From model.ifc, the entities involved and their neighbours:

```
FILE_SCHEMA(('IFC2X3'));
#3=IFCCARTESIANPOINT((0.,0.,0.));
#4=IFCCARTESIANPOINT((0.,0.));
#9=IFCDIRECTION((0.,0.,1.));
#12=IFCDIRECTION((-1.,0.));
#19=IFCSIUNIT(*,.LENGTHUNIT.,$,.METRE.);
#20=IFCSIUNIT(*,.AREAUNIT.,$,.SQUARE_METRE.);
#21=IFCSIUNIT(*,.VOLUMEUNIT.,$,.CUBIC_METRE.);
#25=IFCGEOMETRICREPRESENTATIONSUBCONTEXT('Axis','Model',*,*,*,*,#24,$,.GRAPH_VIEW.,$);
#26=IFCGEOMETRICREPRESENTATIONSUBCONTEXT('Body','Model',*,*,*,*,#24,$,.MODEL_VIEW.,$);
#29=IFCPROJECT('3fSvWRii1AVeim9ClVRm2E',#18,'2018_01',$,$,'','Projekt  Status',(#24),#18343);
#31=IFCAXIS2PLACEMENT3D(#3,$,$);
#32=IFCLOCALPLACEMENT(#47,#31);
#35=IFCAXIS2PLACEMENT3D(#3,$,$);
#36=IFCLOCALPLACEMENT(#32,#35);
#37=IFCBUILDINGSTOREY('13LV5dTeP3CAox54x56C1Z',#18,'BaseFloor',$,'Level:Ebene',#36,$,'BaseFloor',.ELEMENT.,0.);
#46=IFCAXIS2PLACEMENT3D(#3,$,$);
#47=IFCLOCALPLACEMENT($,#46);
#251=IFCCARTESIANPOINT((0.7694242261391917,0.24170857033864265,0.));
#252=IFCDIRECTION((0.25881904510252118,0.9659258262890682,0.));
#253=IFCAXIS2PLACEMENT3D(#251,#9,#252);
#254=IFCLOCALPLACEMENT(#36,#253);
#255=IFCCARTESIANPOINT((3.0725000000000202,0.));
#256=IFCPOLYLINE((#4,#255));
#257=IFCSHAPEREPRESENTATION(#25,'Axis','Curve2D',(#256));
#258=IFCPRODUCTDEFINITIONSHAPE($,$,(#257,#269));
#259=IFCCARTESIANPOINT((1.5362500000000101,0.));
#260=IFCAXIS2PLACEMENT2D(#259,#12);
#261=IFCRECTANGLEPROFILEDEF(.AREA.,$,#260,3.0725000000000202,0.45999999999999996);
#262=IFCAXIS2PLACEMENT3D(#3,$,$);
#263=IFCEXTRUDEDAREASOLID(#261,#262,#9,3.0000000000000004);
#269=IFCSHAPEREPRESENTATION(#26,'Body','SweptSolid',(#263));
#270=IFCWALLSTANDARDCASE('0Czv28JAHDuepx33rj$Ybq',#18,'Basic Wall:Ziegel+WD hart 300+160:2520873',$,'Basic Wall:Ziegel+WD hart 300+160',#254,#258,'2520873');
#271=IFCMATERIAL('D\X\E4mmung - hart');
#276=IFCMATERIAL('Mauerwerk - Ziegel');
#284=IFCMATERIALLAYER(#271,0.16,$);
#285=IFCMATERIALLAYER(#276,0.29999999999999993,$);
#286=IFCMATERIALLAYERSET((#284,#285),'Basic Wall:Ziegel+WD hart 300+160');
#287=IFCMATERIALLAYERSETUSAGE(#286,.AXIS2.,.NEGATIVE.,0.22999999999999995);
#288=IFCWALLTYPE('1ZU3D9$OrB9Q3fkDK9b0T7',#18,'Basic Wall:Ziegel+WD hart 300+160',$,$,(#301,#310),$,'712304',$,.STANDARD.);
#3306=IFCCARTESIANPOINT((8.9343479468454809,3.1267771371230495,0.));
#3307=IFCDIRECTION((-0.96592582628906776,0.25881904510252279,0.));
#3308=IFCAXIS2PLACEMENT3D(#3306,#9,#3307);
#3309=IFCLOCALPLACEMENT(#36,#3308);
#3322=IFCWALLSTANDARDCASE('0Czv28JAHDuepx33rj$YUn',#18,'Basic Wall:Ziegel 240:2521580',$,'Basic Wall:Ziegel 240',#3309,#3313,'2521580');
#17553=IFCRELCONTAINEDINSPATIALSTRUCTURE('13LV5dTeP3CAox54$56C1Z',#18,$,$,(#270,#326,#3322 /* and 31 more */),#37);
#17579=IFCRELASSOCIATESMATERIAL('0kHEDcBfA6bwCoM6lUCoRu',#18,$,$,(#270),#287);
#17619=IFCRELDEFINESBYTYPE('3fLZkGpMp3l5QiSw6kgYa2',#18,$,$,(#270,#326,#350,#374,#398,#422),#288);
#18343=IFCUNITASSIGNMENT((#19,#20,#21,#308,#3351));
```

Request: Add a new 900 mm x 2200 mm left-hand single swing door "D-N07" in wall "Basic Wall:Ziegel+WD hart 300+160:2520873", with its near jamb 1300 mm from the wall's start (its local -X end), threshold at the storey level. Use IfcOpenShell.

```python
import numpy as np
import ifcopenshell
import ifcopenshell.api.feature
import ifcopenshell.api.geometry
import ifcopenshell.api.root
import ifcopenshell.api.spatial
import ifcopenshell.api.type
import ifcopenshell.geom
import ifcopenshell.util.element
import ifcopenshell.util.placement
import ifcopenshell.util.representation
import ifcopenshell.util.shape
import ifcopenshell.util.unit

model = ifcopenshell.open("model.ifc")
unit_scale = ifcopenshell.util.unit.calculate_unit_scale(model)
settings = ifcopenshell.geom.settings()


def volume(element):
    """Net volume in cubic metres, openings subtracted."""
    shape = ifcopenshell.geom.create_shape(settings, element)
    return ifcopenshell.util.shape.get_volume(shape.geometry)


wall = model.by_guid("0Czv28JAHDuepx33rj$Ybq")
storey = ifcopenshell.util.element.get_container(wall, ifc_class="IfcBuildingStorey")
context = ifcopenshell.util.representation.get_context(model, "Model", "Body", "MODEL_VIEW")
before = volume(wall)

width, height, from_end, sill = 0.9, 2.2, 1.3, 0.0  # metres

# The wall runs along its own X axis, and the end named is its -X end.
wall_shape = ifcopenshell.geom.create_shape(settings, wall)
x, y, z = ifcopenshell.util.shape.get_vertices(wall_shape.geometry).T
start = x.min() + from_end
face, thickness = float(y.min()), float(y.max() - y.min())
wall_matrix = ifcopenshell.util.placement.get_local_placement(wall.ObjectPlacement)
level = ifcopenshell.util.placement.get_local_placement(storey.ObjectPlacement)[2, 3]


def in_wall(x, y):
    """Placement at x, y metres in the wall's axes, at sill height."""
    matrix = wall_matrix.copy()
    matrix[:, 3] = wall_matrix @ np.array([x / unit_scale, y / unit_scale, 0.0, 1.0])
    matrix[2, 3] = level + sill / unit_scale
    return matrix


# Opening: a box that overshoots both wall faces by 50 mm.
opening = ifcopenshell.api.root.create_entity(model, ifc_class="IfcOpeningElement")
box = ifcopenshell.api.geometry.add_wall_representation(
    model, context=context, length=width, height=height, thickness=thickness + 0.1
)
ifcopenshell.api.geometry.assign_representation(model, product=opening, representation=box)
ifcopenshell.api.geometry.edit_object_placement(model, product=opening, matrix=in_wall(start, face - 0.05), is_si=False)
ifcopenshell.api.feature.add_feature(model, feature=opening, element=wall)

door = ifcopenshell.api.root.create_entity(model, ifc_class="IfcDoor", name="D-N07")
door.OverallWidth, door.OverallHeight = width / unit_scale, height / unit_scale
body = ifcopenshell.api.geometry.add_door_representation(
    model,
    context=context,
    overall_width=door.OverallWidth,
    overall_height=door.OverallHeight,
    operation_type="SINGLE_SWING_LEFT",
    lining_properties={"LiningDepth": thickness / unit_scale, "ThresholdDepth": thickness / unit_scale},
)
ifcopenshell.api.geometry.assign_representation(model, product=door, representation=body)
ifcopenshell.api.spatial.assign_container(model, products=[door], relating_structure=storey)
fills = ifcopenshell.api.feature.add_filling(model, opening=opening, element=door)
fills.OwnerHistory = door.OwnerHistory  # required in IFC2X3

# IFC2X3 keeps the operation on the door style.
style = ifcopenshell.api.root.create_entity(model, ifc_class="IfcDoorStyle", name="D-N07")
style.OperationType, style.ConstructionType = "SINGLE_SWING_LEFT", "NOTDEFINED"
style.ParameterTakesPrecedence = style.Sizeable = False
ifcopenshell.api.type.assign_type(model, related_objects=[door], relating_type=style)

# The lining spans the wall, so the door starts at the wall face.
ifcopenshell.api.geometry.edit_object_placement(model, product=door, matrix=in_wall(start, face), is_si=False)

after = volume(wall)

print(f"wall volume {before:.3f} -> {after:.3f} m3")

model.write("model_rev.ifc")
```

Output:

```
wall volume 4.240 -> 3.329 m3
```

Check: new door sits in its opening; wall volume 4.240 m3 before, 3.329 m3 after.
